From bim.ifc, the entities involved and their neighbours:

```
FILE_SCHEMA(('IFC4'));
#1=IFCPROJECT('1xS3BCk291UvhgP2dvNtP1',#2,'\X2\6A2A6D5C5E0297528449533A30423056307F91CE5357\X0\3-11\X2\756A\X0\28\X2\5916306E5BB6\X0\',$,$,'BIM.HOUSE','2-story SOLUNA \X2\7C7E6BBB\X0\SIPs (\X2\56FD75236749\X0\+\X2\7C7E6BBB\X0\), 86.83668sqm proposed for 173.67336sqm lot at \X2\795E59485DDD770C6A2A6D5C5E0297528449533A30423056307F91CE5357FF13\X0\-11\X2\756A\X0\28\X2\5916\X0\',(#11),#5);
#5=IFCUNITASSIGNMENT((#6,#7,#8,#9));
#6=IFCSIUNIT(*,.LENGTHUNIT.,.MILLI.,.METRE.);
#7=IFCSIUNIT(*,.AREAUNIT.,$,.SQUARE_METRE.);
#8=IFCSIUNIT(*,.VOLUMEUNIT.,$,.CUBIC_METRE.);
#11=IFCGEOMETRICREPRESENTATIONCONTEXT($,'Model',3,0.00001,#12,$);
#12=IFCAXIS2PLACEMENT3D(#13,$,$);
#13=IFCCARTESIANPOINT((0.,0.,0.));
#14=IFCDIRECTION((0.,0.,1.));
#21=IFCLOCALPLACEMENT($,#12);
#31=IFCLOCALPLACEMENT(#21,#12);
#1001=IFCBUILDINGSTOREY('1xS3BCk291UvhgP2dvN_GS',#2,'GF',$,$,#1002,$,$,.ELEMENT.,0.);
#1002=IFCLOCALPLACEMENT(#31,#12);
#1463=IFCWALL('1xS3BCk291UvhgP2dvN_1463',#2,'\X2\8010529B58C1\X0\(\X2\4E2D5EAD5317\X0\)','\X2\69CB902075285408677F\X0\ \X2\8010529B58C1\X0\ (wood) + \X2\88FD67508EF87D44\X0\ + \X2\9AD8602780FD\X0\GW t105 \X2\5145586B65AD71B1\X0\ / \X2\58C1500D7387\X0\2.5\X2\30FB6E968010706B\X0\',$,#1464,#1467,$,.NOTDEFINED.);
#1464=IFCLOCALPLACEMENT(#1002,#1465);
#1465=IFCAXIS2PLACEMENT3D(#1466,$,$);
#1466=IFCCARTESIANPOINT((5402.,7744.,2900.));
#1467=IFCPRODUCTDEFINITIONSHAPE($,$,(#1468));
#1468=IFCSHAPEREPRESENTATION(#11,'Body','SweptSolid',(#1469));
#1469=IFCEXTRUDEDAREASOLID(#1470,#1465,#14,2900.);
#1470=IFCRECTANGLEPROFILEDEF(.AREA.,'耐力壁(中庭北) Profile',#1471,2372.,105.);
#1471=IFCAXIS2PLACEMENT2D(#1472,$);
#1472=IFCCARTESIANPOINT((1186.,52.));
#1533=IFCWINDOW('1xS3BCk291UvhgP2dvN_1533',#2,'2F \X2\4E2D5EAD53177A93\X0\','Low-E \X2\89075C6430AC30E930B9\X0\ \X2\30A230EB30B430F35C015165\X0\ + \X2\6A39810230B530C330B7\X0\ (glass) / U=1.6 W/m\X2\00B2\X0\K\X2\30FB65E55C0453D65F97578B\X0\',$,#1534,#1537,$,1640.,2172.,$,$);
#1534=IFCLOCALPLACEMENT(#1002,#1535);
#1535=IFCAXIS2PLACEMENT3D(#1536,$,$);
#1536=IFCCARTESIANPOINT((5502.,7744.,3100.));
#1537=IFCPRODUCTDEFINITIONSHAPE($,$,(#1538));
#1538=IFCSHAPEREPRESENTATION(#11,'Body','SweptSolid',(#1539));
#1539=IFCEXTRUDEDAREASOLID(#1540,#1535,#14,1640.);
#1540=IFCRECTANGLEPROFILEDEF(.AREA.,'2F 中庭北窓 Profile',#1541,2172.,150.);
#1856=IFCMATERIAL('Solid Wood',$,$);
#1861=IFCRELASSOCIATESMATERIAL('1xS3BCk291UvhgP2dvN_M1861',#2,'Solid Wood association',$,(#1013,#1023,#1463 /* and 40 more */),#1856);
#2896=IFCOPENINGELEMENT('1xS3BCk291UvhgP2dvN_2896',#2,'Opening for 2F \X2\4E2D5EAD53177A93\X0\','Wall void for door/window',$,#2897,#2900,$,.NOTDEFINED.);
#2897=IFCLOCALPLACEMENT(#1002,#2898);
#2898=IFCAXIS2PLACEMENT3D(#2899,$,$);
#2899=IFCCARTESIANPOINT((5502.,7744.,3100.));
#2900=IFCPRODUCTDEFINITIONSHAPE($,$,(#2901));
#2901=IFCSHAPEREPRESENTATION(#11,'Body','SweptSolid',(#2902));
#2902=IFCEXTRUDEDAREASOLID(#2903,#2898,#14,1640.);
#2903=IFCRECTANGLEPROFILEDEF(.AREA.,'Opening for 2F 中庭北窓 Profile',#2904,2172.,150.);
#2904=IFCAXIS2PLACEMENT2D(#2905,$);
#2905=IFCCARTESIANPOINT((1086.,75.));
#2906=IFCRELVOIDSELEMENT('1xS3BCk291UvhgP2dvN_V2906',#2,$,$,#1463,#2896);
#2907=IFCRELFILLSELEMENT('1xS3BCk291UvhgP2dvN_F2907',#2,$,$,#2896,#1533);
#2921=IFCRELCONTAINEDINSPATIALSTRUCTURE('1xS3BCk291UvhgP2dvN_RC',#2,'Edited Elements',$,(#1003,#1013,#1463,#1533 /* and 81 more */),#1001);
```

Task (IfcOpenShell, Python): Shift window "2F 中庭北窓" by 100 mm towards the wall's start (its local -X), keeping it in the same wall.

```python
import ifcopenshell
import ifcopenshell.api.geometry
import ifcopenshell.util.placement
import ifcopenshell.util.unit

model = ifcopenshell.open("bim.ifc")
unit_scale = ifcopenshell.util.unit.calculate_unit_scale(model)

window = model.by_guid("1xS3BCk291UvhgP2dvN_1533")
opening = window.FillsVoids[0].RelatingOpeningElement
wall = opening.VoidsElements[0].RelatingBuildingElement

wall_matrix = ifcopenshell.util.placement.get_local_placement(wall.ObjectPlacement)
shift = wall_matrix[:3, 0] * -0.1 / unit_scale
before = ifcopenshell.util.placement.get_local_placement(window.ObjectPlacement)[:3, 3].copy()

# The window is not placed relative to its opening, so move both.
for product in (opening, window):
    matrix = ifcopenshell.util.placement.get_local_placement(product.ObjectPlacement)
    matrix[:3, 3] += shift
    ifcopenshell.api.geometry.edit_object_placement(model, product=product, matrix=matrix, is_si=False)

after = ifcopenshell.util.placement.get_local_placement(window.ObjectPlacement)[:3, 3]
print("window moved by", (after - before).round(3) + 0.0)

model.write("bim_edited.ifc")
```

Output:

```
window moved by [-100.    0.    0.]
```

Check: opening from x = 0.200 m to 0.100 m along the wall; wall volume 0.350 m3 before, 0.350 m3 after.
